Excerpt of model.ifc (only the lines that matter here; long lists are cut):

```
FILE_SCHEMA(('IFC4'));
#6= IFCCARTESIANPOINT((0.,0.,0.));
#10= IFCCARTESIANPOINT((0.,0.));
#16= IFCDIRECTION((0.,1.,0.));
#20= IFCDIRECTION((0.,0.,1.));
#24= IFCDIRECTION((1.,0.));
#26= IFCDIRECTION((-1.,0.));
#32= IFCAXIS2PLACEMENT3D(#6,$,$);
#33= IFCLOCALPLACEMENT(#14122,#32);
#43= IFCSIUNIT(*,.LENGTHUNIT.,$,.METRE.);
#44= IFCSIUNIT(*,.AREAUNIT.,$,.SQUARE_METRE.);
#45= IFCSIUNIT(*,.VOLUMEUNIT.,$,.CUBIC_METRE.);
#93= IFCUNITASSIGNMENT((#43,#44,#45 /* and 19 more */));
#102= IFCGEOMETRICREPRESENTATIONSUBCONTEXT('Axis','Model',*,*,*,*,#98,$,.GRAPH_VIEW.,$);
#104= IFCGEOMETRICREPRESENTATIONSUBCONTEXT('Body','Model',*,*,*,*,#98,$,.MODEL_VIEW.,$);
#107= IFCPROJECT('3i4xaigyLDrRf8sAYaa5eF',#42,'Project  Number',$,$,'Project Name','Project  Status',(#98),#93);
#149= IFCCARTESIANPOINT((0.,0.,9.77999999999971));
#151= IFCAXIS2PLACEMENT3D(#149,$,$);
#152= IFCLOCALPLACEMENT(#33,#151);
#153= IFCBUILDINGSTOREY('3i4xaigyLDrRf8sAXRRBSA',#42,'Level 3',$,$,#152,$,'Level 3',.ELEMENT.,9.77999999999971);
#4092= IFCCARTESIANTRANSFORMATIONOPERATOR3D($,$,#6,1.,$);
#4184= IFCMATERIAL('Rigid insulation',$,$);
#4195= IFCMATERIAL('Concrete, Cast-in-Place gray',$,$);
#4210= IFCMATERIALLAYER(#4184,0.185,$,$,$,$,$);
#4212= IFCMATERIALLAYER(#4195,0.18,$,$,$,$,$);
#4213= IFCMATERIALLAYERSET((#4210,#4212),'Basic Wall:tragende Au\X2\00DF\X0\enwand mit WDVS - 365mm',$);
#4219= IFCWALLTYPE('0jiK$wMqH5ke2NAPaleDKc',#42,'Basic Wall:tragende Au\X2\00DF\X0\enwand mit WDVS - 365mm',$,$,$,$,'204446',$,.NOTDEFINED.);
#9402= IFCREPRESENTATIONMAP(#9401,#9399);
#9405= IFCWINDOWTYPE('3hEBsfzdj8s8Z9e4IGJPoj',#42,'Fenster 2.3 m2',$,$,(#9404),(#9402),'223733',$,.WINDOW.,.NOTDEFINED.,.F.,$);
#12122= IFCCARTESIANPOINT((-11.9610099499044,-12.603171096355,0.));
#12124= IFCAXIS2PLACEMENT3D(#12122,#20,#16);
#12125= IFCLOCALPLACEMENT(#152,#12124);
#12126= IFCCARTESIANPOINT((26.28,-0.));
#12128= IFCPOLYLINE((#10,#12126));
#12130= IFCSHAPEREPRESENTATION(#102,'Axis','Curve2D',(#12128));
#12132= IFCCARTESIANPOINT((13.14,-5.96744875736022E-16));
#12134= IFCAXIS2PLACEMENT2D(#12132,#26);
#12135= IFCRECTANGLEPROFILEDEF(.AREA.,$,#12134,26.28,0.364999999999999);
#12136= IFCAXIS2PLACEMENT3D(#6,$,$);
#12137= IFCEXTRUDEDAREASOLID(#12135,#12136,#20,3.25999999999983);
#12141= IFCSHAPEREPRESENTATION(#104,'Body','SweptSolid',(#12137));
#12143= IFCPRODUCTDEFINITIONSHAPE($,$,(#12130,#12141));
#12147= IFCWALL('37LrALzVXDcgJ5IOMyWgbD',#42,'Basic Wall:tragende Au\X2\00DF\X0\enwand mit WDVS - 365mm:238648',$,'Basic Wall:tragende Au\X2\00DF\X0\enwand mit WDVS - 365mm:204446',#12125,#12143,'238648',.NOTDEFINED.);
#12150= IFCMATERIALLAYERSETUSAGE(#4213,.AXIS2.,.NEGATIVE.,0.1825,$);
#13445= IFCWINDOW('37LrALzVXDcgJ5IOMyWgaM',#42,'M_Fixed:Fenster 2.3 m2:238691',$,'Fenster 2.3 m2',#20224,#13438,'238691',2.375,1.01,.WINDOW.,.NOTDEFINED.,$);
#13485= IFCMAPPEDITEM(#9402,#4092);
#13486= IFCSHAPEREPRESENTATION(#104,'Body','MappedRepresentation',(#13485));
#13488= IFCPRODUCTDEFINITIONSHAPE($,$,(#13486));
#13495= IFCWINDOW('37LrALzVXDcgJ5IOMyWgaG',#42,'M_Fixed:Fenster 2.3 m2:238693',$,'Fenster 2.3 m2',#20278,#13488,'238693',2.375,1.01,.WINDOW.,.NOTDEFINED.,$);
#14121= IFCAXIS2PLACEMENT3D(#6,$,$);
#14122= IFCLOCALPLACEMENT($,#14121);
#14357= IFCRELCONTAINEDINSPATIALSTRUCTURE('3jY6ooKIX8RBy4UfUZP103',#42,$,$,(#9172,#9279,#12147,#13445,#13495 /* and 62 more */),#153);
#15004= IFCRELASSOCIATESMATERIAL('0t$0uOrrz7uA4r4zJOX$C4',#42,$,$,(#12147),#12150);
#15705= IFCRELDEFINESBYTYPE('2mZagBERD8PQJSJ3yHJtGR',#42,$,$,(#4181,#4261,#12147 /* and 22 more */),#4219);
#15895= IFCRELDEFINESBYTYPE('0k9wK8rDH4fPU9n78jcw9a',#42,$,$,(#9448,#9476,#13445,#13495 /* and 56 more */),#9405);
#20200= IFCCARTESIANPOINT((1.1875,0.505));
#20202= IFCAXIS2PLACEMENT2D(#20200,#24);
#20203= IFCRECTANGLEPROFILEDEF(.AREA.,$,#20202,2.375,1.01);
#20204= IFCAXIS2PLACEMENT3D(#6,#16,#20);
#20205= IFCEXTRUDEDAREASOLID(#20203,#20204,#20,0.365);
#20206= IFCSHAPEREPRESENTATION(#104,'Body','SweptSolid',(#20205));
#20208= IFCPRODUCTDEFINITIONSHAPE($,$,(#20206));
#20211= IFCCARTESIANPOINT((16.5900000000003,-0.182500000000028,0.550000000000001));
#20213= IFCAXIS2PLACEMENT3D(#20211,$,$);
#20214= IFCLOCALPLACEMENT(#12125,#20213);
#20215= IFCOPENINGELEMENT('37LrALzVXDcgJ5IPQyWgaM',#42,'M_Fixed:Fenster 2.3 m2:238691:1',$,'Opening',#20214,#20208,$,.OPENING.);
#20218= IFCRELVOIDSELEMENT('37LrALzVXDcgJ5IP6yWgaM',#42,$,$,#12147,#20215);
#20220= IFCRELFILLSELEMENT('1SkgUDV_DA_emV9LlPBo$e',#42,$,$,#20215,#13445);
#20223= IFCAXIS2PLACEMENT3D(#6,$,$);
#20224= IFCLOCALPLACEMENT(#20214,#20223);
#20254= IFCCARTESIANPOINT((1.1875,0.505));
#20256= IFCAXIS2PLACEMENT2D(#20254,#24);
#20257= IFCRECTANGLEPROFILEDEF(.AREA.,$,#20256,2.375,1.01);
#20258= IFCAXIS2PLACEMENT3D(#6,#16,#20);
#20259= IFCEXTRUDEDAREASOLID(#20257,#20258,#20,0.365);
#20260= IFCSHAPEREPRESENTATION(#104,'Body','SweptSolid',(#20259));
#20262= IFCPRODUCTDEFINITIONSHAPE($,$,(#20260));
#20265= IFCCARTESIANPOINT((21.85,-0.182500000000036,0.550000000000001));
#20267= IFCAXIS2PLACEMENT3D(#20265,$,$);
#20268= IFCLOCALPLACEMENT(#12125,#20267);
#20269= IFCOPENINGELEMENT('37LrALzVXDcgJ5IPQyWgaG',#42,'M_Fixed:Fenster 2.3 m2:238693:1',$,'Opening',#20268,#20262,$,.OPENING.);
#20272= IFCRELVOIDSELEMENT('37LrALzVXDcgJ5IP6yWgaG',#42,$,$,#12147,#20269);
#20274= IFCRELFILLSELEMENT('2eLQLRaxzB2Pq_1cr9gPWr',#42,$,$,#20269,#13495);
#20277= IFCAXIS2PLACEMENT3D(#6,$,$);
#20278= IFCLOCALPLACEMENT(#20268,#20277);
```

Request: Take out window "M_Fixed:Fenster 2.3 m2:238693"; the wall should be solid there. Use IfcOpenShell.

```python
import ifcopenshell
import ifcopenshell.api.feature
import ifcopenshell.api.root
import ifcopenshell.geom
import ifcopenshell.util.shape

model = ifcopenshell.open("model.ifc")
settings = ifcopenshell.geom.settings()


def volume(element):
    """Net volume in cubic metres, openings subtracted."""
    shape = ifcopenshell.geom.create_shape(settings, element)
    return ifcopenshell.util.shape.get_volume(shape.geometry)


window = model.by_id(13495)
opening = window.FillsVoids[0].RelatingOpeningElement
wall = opening.VoidsElements[0].RelatingBuildingElement
before = volume(wall)

ifcopenshell.api.root.remove_product(model, product=window)
ifcopenshell.api.feature.remove_feature(model, feature=opening)

after = volume(wall)

print(f"wall volume {before:.3f} -> {after:.3f} m3")

model.write("model_updated.ifc")
```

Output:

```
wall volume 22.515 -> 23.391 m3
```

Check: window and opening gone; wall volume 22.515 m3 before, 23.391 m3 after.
